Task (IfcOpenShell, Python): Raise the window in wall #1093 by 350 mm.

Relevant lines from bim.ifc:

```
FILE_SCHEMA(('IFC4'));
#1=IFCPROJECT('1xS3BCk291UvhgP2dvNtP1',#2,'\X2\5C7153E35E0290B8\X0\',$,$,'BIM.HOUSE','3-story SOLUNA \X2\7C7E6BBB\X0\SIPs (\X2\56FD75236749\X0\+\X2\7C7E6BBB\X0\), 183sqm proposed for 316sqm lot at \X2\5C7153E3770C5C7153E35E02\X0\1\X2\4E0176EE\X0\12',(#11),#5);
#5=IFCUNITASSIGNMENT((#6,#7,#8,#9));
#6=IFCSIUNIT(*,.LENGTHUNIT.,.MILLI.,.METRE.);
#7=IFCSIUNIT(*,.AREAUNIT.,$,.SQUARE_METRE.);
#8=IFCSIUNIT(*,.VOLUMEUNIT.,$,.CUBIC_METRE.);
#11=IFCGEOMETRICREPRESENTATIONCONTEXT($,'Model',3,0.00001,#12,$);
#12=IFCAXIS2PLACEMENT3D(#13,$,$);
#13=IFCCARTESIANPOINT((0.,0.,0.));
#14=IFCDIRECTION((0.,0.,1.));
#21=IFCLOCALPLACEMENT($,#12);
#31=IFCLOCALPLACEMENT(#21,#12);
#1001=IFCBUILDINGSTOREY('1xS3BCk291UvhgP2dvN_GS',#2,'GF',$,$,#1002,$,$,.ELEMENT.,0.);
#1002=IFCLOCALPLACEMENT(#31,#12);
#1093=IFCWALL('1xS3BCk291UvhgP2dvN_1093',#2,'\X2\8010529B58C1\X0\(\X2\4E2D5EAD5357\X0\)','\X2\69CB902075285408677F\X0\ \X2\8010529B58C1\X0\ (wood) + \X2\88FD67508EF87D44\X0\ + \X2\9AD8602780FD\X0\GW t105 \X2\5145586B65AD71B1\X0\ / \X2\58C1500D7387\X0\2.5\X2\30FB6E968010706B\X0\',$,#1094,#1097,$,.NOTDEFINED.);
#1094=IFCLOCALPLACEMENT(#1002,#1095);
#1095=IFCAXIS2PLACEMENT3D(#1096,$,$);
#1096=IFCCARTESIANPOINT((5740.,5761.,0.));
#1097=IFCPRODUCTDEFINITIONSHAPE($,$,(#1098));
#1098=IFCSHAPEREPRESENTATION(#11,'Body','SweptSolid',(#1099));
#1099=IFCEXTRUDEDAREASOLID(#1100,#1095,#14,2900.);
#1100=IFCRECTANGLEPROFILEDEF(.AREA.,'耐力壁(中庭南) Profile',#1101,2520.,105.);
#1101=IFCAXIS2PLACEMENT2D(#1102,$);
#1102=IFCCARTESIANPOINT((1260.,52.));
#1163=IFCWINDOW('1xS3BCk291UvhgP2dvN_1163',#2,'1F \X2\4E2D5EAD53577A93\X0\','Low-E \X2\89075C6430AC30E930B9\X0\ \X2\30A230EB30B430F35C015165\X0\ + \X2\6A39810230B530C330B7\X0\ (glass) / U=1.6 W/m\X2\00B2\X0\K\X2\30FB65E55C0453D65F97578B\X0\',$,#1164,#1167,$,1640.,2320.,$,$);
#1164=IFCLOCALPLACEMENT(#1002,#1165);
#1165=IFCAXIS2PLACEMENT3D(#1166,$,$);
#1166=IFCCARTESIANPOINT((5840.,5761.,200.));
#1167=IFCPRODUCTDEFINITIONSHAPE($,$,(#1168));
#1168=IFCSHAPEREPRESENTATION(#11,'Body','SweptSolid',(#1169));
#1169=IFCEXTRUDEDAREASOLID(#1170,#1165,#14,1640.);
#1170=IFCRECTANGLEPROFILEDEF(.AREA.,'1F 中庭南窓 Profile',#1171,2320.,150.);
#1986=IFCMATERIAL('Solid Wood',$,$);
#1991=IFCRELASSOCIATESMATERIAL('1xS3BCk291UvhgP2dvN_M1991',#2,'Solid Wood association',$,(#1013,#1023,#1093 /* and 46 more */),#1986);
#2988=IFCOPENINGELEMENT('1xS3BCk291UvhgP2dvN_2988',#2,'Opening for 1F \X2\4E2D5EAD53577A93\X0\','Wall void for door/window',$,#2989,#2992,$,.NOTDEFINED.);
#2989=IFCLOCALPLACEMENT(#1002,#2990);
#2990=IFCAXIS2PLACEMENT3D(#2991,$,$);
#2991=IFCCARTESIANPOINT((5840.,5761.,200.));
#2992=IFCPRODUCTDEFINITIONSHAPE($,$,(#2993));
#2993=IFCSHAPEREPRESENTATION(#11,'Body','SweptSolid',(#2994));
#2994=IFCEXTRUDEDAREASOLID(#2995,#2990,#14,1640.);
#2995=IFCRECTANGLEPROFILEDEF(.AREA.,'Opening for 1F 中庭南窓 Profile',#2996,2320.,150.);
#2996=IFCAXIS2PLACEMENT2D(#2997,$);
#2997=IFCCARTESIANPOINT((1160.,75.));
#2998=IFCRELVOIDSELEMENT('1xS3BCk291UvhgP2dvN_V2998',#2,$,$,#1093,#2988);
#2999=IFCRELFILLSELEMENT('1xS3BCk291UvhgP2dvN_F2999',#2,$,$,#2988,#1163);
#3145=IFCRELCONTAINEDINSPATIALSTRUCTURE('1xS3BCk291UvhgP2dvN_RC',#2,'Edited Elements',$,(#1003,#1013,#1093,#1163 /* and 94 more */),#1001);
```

```python
import numpy as np
import ifcopenshell
import ifcopenshell.api.geometry
import ifcopenshell.util.placement
import ifcopenshell.util.unit

model = ifcopenshell.open("bim.ifc")
unit_scale = ifcopenshell.util.unit.calculate_unit_scale(model)

window = model.by_id(1163)
opening = window.FillsVoids[0].RelatingOpeningElement
dz = 350.0

shift = np.array([0.0, 0.0, dz])
# The window is not placed relative to its opening, so move both.
for product in (opening, window):
    matrix = ifcopenshell.util.placement.get_local_placement(product.ObjectPlacement)
    matrix[:3, 3] += shift
    ifcopenshell.api.geometry.edit_object_placement(model, product=product, matrix=matrix, is_si=False)

print(f"moved by {dz * unit_scale:+.3f} m")

model.write("bim_edited.ifc")
```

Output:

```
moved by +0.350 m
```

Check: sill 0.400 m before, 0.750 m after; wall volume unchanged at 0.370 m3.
